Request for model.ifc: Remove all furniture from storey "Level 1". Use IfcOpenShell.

First a look at what the model holds.

```python
import ifcopenshell
import ifcopenshell.util.element

model = ifcopenshell.open("model.ifc")
print(model.schema)
storey = next(s for s in model.by_type("IfcBuildingStorey") if s.Name == "Level 1")
furniture = [e for e in ifcopenshell.util.element.get_decomposition(storey) if e.is_a("IfcFurnishingElement")]
seen = {}
for e in furniture:
    element_type = ifcopenshell.util.element.get_type(e)
    name = element_type.Name if element_type not in (None, e) else None
    seen[name] = seen.get(name, 0) + 1
for name, count in sorted(seen.items(), key=str):
    print(count, "x", name)
```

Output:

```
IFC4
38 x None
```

```python
import ifcopenshell
import ifcopenshell.api.root
import ifcopenshell.util.element

model = ifcopenshell.open("model.ifc")

storey = next(s for s in model.by_type("IfcBuildingStorey") if s.Name == "Level 1")
furniture = [e for e in ifcopenshell.util.element.get_decomposition(storey) if e.is_a("IfcFurnishingElement")]

for e in furniture:
    ifcopenshell.api.root.remove_product(model, product=e)
print(len(furniture), "removed")

model.write("model_updated.ifc")
```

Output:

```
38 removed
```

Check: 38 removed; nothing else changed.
